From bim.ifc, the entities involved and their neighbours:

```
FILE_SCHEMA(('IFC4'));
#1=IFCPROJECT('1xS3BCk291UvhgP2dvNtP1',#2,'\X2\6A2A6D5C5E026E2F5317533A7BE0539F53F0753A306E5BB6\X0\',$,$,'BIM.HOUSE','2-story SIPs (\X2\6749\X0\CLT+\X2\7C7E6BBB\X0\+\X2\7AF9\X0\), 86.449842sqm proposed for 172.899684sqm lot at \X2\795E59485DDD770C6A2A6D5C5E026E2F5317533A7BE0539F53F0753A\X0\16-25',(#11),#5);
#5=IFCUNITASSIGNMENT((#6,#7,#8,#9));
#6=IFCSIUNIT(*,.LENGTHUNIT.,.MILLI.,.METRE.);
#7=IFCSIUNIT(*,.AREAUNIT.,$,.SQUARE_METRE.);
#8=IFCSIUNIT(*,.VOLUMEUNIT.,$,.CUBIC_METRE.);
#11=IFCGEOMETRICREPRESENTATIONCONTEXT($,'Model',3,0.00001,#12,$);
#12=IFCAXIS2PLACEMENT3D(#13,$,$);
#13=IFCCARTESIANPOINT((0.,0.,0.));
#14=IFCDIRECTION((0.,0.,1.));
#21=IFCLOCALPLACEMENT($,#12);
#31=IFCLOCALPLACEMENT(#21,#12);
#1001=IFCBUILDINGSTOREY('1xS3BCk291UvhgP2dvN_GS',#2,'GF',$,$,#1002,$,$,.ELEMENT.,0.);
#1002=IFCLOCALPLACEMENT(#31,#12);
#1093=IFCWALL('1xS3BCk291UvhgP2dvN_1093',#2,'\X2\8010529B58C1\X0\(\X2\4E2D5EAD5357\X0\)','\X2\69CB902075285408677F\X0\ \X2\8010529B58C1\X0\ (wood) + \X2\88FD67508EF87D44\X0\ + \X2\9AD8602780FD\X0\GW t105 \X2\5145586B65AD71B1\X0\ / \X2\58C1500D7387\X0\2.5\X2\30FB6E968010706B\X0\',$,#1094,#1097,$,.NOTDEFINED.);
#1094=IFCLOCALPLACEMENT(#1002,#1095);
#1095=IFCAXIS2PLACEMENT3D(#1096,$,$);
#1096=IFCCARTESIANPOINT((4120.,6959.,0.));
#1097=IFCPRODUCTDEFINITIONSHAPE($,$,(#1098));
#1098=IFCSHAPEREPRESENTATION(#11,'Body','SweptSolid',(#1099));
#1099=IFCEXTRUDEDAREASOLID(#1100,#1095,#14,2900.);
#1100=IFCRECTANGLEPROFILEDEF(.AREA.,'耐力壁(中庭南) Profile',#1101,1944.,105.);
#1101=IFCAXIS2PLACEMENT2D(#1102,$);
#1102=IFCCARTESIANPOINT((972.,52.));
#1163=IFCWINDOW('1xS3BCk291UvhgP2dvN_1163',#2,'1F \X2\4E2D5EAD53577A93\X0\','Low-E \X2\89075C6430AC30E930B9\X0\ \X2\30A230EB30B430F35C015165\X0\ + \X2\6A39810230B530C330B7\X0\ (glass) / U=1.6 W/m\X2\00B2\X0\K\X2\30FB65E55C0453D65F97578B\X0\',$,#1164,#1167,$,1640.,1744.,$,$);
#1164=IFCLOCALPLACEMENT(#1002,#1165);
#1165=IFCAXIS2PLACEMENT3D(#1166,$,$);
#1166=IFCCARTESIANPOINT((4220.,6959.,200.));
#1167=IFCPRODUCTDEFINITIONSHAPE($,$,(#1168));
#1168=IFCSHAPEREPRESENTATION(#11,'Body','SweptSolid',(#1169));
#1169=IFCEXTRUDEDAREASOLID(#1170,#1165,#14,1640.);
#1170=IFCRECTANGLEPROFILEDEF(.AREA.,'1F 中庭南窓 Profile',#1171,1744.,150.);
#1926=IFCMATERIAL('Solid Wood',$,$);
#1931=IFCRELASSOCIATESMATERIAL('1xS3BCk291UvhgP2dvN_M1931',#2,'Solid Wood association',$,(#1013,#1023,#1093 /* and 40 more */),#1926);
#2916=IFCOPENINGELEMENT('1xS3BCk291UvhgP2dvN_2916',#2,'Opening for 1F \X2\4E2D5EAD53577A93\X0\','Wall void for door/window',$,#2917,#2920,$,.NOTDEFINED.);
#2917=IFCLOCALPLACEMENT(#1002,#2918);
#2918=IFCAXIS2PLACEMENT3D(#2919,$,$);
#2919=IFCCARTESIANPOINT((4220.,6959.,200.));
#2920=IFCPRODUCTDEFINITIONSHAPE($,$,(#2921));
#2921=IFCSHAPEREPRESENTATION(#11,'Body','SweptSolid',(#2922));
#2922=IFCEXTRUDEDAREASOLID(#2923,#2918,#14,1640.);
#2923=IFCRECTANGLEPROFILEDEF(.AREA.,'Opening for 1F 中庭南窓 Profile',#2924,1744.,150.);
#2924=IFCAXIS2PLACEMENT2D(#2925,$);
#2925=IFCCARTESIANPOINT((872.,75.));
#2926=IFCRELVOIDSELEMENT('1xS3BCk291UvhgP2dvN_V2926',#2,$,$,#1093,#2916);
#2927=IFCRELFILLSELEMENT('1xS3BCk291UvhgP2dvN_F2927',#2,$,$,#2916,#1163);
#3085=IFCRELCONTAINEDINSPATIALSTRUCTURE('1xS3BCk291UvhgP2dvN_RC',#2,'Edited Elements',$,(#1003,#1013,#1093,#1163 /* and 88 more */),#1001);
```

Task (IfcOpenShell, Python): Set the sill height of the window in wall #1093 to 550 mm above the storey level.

```python
import numpy as np
import ifcopenshell
import ifcopenshell.api.geometry
import ifcopenshell.geom
import ifcopenshell.util.element
import ifcopenshell.util.placement
import ifcopenshell.util.shape
import ifcopenshell.util.unit

model = ifcopenshell.open("bim.ifc")
unit_scale = ifcopenshell.util.unit.calculate_unit_scale(model)

window = model.by_guid("1xS3BCk291UvhgP2dvN_1163")
opening = window.FillsVoids[0].RelatingOpeningElement
storey = ifcopenshell.util.element.get_container(window, ifc_class="IfcBuildingStorey")
level = ifcopenshell.util.placement.get_local_placement(storey.ObjectPlacement)[2, 3]

# The opening's origin need not be at the sill, so measure its lowest point.
shape = ifcopenshell.geom.create_shape(ifcopenshell.geom.settings(), opening)
bottom = ifcopenshell.util.shape.get_shape_bottom_elevation(shape, shape.geometry) / unit_scale
dz = level + 550.0 - bottom

shift = np.array([0.0, 0.0, dz])
# The window is not placed relative to its opening, so move both.
for product in (opening, window):
    matrix = ifcopenshell.util.placement.get_local_placement(product.ObjectPlacement)
    matrix[:3, 3] += shift
    ifcopenshell.api.geometry.edit_object_placement(model, product=product, matrix=matrix, is_si=False)

print(f"moved by {dz * unit_scale:+.3f} m")

model.write("bim_updated.ifc")
```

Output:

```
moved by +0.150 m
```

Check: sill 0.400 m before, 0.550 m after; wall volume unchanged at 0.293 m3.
